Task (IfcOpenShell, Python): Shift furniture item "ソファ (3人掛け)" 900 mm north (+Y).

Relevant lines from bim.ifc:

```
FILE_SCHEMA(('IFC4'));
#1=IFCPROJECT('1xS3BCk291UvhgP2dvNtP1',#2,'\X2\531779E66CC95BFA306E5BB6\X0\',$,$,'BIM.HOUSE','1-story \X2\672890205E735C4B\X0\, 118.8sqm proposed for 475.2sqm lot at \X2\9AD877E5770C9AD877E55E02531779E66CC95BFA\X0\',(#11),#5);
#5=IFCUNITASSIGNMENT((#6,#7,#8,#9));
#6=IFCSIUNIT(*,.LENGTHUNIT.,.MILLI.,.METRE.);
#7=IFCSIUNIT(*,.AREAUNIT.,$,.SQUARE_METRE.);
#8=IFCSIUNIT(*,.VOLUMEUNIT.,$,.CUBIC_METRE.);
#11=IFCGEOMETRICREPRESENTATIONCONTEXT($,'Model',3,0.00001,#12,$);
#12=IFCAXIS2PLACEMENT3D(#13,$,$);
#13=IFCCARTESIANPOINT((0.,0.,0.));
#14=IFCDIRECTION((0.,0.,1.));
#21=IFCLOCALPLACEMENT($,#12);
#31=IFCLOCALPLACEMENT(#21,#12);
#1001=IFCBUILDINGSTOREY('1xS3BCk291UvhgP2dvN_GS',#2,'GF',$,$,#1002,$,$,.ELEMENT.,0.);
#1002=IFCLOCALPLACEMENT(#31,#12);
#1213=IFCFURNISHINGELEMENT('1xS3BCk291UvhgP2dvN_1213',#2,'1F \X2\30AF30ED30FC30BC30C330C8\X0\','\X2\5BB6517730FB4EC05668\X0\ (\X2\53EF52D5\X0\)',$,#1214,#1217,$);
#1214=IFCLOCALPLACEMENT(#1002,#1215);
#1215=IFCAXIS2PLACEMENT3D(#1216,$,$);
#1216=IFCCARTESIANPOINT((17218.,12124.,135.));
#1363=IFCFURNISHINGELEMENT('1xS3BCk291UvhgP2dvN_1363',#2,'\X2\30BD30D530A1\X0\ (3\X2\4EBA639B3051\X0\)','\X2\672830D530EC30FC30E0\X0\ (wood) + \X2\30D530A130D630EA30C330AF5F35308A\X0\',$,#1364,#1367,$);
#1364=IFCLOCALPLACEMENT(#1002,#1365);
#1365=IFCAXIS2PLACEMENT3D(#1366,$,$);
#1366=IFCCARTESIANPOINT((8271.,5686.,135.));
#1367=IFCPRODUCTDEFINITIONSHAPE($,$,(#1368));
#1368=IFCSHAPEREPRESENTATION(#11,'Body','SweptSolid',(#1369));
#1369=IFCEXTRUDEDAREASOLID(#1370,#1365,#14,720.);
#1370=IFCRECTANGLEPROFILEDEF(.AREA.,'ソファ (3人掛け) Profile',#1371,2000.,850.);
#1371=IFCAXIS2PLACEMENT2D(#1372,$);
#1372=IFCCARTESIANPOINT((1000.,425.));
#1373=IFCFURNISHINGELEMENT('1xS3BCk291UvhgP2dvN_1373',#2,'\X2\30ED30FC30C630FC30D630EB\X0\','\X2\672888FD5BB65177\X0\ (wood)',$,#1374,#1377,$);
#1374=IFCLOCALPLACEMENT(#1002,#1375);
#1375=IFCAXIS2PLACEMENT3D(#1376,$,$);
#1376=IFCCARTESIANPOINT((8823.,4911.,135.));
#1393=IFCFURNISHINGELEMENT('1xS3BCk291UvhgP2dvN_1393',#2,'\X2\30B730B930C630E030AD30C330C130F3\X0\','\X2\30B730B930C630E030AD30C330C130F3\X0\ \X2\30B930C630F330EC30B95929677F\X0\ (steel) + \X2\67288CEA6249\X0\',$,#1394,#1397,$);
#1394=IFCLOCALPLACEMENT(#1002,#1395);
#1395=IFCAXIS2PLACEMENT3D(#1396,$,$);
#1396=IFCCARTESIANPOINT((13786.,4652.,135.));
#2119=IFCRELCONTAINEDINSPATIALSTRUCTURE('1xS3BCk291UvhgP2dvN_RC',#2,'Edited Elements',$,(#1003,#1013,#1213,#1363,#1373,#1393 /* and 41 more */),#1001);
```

```python
import ifcopenshell
import ifcopenshell.api.geometry
import ifcopenshell.util.placement
import ifcopenshell.util.unit

model = ifcopenshell.open("bim.ifc")
unit_scale = ifcopenshell.util.unit.calculate_unit_scale(model)

item = model.by_guid("1xS3BCk291UvhgP2dvN_1363")
matrix = ifcopenshell.util.placement.get_local_placement(item.ObjectPlacement)
matrix[1, 3] += 0.9 / unit_scale
ifcopenshell.api.geometry.edit_object_placement(model, product=item, matrix=matrix, is_si=False)

print(ifcopenshell.util.placement.get_local_placement(item.ObjectPlacement).round(3) + 0.0)

model.write("bim_v2.ifc")
```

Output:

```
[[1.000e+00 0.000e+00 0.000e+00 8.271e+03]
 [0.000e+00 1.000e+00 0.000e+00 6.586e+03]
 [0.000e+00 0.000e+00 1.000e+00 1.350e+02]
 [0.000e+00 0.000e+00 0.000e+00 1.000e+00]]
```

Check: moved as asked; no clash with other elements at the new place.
